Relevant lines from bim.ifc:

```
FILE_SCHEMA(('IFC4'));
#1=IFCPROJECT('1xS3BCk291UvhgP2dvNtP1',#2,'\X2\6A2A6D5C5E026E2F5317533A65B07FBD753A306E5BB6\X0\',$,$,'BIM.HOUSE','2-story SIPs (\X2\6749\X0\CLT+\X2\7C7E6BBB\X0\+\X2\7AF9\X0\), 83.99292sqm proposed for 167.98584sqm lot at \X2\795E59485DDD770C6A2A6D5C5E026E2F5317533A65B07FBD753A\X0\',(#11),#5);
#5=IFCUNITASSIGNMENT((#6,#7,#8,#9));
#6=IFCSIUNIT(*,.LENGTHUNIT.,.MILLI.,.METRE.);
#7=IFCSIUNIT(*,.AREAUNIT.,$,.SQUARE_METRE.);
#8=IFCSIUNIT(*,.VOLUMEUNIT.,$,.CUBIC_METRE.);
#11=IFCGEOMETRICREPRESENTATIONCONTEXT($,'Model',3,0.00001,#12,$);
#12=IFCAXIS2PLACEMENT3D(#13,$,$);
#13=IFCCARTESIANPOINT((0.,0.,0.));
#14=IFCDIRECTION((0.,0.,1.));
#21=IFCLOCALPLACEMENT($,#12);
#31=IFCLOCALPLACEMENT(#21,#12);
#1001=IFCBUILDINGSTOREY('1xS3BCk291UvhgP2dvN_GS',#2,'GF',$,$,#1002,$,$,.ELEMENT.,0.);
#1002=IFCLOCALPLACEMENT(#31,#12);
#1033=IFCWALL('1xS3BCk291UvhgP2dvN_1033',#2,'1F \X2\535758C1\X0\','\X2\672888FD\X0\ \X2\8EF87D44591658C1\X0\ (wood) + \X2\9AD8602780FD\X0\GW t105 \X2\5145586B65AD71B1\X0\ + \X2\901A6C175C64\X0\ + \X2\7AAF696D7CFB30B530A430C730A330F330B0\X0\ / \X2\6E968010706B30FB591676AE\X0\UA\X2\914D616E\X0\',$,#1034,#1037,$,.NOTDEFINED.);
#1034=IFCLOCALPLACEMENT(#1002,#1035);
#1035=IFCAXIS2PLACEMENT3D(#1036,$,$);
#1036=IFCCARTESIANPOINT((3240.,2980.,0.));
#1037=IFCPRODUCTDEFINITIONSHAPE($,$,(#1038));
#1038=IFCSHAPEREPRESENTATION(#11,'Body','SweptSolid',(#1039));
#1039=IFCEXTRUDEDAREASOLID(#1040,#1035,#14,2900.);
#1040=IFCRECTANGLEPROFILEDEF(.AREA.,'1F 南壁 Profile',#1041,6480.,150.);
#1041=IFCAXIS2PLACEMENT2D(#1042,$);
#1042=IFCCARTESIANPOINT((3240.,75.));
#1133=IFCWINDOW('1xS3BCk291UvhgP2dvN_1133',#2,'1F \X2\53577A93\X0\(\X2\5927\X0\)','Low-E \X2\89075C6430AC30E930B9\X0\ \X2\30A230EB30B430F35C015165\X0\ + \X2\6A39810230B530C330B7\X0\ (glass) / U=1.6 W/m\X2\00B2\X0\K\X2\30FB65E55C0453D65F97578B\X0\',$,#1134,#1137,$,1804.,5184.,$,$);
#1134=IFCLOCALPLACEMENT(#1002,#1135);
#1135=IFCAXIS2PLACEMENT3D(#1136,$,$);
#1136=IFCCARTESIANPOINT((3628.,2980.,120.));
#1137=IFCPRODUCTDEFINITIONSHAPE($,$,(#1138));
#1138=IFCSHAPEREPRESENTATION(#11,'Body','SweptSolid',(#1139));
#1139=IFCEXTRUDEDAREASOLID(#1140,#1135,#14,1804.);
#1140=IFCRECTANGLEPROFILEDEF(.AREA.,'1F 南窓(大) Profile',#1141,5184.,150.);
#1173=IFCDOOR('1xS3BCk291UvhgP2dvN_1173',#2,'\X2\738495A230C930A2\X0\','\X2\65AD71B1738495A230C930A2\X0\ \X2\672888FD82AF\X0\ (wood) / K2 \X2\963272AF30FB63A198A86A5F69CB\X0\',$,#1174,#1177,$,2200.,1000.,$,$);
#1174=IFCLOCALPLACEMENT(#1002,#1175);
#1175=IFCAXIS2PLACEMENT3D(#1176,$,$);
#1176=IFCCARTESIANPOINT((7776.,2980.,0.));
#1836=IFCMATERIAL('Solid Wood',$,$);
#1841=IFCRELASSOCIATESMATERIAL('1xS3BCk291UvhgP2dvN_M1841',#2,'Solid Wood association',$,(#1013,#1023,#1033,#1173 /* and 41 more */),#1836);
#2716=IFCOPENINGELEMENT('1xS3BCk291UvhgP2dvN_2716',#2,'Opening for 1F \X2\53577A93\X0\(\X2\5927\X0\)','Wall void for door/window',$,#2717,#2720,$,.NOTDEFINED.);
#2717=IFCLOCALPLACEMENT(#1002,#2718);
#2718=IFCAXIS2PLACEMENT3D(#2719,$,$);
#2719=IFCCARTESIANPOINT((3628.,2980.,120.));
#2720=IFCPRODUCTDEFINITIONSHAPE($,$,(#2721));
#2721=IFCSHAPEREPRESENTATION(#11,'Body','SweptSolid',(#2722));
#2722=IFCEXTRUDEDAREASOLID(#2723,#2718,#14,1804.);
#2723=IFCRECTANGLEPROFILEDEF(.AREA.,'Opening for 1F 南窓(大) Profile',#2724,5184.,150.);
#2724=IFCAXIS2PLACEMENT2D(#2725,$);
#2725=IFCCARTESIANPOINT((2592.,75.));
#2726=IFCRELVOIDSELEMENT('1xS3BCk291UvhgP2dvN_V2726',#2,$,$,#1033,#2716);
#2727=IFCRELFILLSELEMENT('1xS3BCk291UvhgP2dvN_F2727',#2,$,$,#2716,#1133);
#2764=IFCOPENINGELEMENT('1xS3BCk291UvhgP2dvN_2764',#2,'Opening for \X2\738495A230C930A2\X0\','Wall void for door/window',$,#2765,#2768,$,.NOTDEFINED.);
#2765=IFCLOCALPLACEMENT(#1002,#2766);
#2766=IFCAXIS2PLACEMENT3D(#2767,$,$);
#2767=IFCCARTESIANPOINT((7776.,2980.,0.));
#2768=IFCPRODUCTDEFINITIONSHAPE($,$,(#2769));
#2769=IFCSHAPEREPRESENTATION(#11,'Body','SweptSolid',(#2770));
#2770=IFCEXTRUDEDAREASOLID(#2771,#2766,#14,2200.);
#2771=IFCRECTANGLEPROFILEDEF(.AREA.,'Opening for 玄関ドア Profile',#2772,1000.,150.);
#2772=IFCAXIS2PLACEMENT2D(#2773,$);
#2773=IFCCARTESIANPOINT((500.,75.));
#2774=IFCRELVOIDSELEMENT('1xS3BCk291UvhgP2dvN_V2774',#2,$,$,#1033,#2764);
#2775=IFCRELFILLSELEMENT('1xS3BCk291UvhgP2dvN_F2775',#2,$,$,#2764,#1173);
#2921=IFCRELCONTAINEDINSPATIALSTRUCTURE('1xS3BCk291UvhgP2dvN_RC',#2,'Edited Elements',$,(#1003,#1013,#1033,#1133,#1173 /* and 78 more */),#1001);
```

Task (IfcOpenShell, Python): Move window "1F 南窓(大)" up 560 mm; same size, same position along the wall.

```python
import numpy as np
import ifcopenshell
import ifcopenshell.api.geometry
import ifcopenshell.util.placement
import ifcopenshell.util.unit

model = ifcopenshell.open("bim.ifc")
unit_scale = ifcopenshell.util.unit.calculate_unit_scale(model)

window = model.by_guid("1xS3BCk291UvhgP2dvN_1133")
opening = window.FillsVoids[0].RelatingOpeningElement
dz = 0.56 / unit_scale

shift = np.array([0.0, 0.0, dz])
# The window is not placed relative to its opening, so move both.
for product in (opening, window):
    matrix = ifcopenshell.util.placement.get_local_placement(product.ObjectPlacement)
    matrix[:3, 3] += shift
    ifcopenshell.api.geometry.edit_object_placement(model, product=product, matrix=matrix, is_si=False)

print(f"moved by {dz * unit_scale:+.3f} m")

model.write("bim_updated.ifc")
```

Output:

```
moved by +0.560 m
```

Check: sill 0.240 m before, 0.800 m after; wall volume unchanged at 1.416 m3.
